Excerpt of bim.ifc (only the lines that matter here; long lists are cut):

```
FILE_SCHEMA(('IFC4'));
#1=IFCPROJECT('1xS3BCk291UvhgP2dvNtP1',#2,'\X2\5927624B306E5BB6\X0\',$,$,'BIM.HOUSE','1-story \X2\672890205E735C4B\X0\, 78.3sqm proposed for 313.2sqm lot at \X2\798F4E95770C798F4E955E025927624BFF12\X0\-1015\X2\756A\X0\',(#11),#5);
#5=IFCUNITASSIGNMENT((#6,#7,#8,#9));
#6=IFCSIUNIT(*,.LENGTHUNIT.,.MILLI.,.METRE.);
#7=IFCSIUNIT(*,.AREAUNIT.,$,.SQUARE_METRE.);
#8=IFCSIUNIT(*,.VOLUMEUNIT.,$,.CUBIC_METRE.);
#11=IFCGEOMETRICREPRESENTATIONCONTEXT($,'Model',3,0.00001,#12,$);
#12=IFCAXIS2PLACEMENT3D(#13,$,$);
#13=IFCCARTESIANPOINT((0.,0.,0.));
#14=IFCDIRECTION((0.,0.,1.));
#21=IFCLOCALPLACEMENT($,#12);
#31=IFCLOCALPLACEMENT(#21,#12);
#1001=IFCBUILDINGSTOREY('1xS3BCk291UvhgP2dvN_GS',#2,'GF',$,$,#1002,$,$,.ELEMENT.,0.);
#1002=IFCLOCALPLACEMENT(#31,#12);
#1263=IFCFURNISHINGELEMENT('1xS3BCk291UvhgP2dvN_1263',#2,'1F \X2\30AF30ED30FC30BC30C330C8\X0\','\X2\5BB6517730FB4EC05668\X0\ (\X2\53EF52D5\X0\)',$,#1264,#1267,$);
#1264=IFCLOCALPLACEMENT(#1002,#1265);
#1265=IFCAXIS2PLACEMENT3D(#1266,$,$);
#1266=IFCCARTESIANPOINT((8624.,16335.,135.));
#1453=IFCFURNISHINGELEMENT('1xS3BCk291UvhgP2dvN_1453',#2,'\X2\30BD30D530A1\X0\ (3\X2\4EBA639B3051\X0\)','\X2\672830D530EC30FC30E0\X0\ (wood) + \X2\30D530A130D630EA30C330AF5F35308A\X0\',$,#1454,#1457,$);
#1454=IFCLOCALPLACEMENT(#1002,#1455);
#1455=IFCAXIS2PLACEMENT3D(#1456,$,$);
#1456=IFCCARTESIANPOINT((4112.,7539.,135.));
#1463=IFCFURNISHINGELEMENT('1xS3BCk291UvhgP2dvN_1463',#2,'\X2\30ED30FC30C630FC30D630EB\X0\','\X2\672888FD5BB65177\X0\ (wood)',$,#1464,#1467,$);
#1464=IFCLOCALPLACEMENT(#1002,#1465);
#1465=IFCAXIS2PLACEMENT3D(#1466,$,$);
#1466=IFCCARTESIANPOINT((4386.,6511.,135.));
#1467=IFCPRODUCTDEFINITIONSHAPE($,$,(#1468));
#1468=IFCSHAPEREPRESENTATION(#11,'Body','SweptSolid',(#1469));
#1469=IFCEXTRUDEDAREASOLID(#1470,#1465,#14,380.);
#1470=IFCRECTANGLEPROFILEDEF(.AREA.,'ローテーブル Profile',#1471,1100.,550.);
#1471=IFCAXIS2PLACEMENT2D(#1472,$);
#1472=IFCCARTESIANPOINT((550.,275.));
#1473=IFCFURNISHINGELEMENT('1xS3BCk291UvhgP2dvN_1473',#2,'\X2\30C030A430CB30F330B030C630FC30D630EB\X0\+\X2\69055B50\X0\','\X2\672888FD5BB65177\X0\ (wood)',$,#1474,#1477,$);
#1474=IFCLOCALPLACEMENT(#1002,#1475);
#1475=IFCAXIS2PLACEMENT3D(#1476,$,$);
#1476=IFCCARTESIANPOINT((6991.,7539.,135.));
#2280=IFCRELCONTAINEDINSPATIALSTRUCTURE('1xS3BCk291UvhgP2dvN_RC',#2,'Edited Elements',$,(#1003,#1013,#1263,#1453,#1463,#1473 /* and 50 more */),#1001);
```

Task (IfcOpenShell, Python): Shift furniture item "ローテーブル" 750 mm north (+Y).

```python
import ifcopenshell
import ifcopenshell.api.geometry
import ifcopenshell.util.placement
import ifcopenshell.util.unit

model = ifcopenshell.open("bim.ifc")
unit_scale = ifcopenshell.util.unit.calculate_unit_scale(model)

item = model.by_guid("1xS3BCk291UvhgP2dvN_1463")
matrix = ifcopenshell.util.placement.get_local_placement(item.ObjectPlacement)
matrix[1, 3] += 0.75 / unit_scale
ifcopenshell.api.geometry.edit_object_placement(model, product=item, matrix=matrix, is_si=False)

print(ifcopenshell.util.placement.get_local_placement(item.ObjectPlacement).round(3) + 0.0)

model.write("bim_v2.ifc")
```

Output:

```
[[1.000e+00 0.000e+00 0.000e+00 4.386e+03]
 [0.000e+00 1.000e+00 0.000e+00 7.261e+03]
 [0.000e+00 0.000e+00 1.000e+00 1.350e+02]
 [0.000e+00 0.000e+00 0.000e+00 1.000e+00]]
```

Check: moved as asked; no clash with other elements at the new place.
